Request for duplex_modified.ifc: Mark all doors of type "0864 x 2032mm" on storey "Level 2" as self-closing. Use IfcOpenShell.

First a look at what the model holds.

```python
import ifcopenshell
import ifcopenshell.util.element

model = ifcopenshell.open("duplex_modified.ifc")
print(model.schema)
storey = next(s for s in model.by_type("IfcBuildingStorey") if s.Name == "Level 2")
doors = [e for e in ifcopenshell.util.element.get_decomposition(storey) if e.is_a("IfcDoor")]
seen = {}
for e in doors:
    element_type = ifcopenshell.util.element.get_type(e)
    key = (element_type.Name if element_type != e and element_type else None, ifcopenshell.util.element.get_pset(e, "Pset_DoorCommon", "SelfClosing"))
    seen[key] = seen.get(key, 0) + 1
for (name, value), count in sorted(seen.items(), key=str):
    print(count, "x", name, "|", value)
```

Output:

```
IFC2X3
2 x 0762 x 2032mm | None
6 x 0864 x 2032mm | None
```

```python
import ifcopenshell
import ifcopenshell.api.pset
import ifcopenshell.util.element

model = ifcopenshell.open("duplex_modified.ifc")

storey = next(s for s in model.by_type("IfcBuildingStorey") if s.Name == "Level 2")
doors = [e for e in ifcopenshell.util.element.get_decomposition(storey) if e.is_a("IfcDoor")]

count = 0
for e in doors:
    element_type = ifcopenshell.util.element.get_type(e)
    if element_type in (None, e) or element_type.Name != "0864 x 2032mm":
        continue
    # add_pset returns the element's existing set when there is one.
    pset = ifcopenshell.api.pset.add_pset(model, product=e, name="Pset_DoorCommon")
    ifcopenshell.api.pset.edit_pset(model, pset=pset, properties={"SelfClosing": True})
    count += 1

print(count, "doors updated")

model.write("duplex_modified_edited.ifc")
```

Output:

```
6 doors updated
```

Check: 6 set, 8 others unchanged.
